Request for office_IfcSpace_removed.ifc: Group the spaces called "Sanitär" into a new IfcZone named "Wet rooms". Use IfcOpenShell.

First a look at what the model holds.

```python
import ifcopenshell

model = ifcopenshell.open("office_IfcSpace_removed.ifc")
print(model.schema)
seen = {}
for space in model.by_type("IfcSpace"):
    seen[space.LongName] = seen.get(space.LongName, 0) + 1
for name, count in sorted(seen.items(), key=str):
    print(count, "x", name)
print("zones:", [z.Name for z in model.by_type("IfcZone")][:20])
```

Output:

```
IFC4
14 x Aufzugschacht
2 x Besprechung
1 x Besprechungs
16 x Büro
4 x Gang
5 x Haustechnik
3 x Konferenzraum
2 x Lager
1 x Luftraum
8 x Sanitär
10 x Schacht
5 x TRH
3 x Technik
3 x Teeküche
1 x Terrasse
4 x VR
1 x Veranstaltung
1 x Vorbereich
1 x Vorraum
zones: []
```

```python
import ifcopenshell
import ifcopenshell.api.group
import ifcopenshell.api.root

model = ifcopenshell.open("office_IfcSpace_removed.ifc")

names = {"Sanitär"}
spaces = [s for s in model.by_type("IfcSpace") if s.LongName in names]

zone = ifcopenshell.api.root.create_entity(model, ifc_class="IfcZone", name="Wet rooms")
ifcopenshell.api.group.assign_group(model, products=spaces, group=zone)
print(len(spaces), "spaces in", zone.Name)

model.write("office_IfcSpace_removed_updated.ifc")
```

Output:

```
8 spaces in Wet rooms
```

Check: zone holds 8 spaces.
